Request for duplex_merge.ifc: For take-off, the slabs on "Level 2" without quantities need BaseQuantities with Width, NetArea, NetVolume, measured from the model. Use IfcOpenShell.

First a look at what the model holds.

```python
import ifcopenshell
import ifcopenshell.util.element
import ifcopenshell.util.unit

model = ifcopenshell.open("duplex_merge.ifc")
print(model.schema)
for unit_type in ("LENGTHUNIT", "AREAUNIT", "VOLUMEUNIT"):
    print(unit_type, ifcopenshell.util.unit.calculate_unit_scale(model, unit_type))
storey = next(s for s in model.by_type("IfcBuildingStorey") if s.Name == "Level 2")
slabs = [e for e in ifcopenshell.util.element.get_decomposition(storey) if e.is_a("IfcSlab")]
for e in sorted(slabs, key=lambda e: e.id()):
    print(e.id(), e.is_a(), e.Name, list(ifcopenshell.util.element.get_psets(e, qtos_only=True)), sep=" | ")
```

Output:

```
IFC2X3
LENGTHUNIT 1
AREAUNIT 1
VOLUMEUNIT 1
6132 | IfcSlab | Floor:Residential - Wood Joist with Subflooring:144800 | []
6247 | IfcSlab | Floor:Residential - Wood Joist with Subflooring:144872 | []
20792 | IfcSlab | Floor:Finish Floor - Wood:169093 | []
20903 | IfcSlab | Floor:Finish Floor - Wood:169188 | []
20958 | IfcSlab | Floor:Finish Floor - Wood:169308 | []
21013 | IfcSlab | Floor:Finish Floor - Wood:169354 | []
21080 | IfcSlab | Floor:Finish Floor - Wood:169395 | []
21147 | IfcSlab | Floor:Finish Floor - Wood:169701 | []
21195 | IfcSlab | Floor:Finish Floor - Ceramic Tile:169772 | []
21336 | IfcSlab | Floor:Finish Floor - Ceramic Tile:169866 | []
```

```python
import ifcopenshell
import ifcopenshell.api.pset
import ifcopenshell.geom
import ifcopenshell.util.element
import ifcopenshell.util.shape
import ifcopenshell.util.unit

model = ifcopenshell.open("duplex_merge.ifc")
unit_scale = ifcopenshell.util.unit.calculate_unit_scale(model)
area_scale = ifcopenshell.util.unit.calculate_unit_scale(model, "AREAUNIT")
volume_scale = ifcopenshell.util.unit.calculate_unit_scale(model, "VOLUMEUNIT")
settings = ifcopenshell.geom.settings()

storey = next(s for s in model.by_type("IfcBuildingStorey") if s.Name == "Level 2")
slabs = [e for e in ifcopenshell.util.element.get_decomposition(storey) if e.is_a("IfcSlab")]

for e in sorted(slabs, key=lambda e: e.id()):
    if ifcopenshell.util.element.get_psets(e, qtos_only=True, should_inherit=False):
        continue
    # Geometry comes back in metres, in the element's own axes.
    shape = ifcopenshell.geom.create_shape(settings, e)
    values = {
        "Width": ifcopenshell.util.shape.get_z(shape.geometry) / unit_scale,
        "NetArea": ifcopenshell.util.shape.get_footprint_area(shape.geometry) / area_scale,
        "NetVolume": ifcopenshell.util.shape.get_volume(shape.geometry) / volume_scale,
    }
    qto = ifcopenshell.api.pset.add_qto(model, product=e, name="BaseQuantities")
    ifcopenshell.api.pset.edit_qto(model, qto=qto, properties=values)
    print(e.id(), {k: round(v, 3) for k, v in values.items()})

model.write("duplex_merge_v2.ifc")
```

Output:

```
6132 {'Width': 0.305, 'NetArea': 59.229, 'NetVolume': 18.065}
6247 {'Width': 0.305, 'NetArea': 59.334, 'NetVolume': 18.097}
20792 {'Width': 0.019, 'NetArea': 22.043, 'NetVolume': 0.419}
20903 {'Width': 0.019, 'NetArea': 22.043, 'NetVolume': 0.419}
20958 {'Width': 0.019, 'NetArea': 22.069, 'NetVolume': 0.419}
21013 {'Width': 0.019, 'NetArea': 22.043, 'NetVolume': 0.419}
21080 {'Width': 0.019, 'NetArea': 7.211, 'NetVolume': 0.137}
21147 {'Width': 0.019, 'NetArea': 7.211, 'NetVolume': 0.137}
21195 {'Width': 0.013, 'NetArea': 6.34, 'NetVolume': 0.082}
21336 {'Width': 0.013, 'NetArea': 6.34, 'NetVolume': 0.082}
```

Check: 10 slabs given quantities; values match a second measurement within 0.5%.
